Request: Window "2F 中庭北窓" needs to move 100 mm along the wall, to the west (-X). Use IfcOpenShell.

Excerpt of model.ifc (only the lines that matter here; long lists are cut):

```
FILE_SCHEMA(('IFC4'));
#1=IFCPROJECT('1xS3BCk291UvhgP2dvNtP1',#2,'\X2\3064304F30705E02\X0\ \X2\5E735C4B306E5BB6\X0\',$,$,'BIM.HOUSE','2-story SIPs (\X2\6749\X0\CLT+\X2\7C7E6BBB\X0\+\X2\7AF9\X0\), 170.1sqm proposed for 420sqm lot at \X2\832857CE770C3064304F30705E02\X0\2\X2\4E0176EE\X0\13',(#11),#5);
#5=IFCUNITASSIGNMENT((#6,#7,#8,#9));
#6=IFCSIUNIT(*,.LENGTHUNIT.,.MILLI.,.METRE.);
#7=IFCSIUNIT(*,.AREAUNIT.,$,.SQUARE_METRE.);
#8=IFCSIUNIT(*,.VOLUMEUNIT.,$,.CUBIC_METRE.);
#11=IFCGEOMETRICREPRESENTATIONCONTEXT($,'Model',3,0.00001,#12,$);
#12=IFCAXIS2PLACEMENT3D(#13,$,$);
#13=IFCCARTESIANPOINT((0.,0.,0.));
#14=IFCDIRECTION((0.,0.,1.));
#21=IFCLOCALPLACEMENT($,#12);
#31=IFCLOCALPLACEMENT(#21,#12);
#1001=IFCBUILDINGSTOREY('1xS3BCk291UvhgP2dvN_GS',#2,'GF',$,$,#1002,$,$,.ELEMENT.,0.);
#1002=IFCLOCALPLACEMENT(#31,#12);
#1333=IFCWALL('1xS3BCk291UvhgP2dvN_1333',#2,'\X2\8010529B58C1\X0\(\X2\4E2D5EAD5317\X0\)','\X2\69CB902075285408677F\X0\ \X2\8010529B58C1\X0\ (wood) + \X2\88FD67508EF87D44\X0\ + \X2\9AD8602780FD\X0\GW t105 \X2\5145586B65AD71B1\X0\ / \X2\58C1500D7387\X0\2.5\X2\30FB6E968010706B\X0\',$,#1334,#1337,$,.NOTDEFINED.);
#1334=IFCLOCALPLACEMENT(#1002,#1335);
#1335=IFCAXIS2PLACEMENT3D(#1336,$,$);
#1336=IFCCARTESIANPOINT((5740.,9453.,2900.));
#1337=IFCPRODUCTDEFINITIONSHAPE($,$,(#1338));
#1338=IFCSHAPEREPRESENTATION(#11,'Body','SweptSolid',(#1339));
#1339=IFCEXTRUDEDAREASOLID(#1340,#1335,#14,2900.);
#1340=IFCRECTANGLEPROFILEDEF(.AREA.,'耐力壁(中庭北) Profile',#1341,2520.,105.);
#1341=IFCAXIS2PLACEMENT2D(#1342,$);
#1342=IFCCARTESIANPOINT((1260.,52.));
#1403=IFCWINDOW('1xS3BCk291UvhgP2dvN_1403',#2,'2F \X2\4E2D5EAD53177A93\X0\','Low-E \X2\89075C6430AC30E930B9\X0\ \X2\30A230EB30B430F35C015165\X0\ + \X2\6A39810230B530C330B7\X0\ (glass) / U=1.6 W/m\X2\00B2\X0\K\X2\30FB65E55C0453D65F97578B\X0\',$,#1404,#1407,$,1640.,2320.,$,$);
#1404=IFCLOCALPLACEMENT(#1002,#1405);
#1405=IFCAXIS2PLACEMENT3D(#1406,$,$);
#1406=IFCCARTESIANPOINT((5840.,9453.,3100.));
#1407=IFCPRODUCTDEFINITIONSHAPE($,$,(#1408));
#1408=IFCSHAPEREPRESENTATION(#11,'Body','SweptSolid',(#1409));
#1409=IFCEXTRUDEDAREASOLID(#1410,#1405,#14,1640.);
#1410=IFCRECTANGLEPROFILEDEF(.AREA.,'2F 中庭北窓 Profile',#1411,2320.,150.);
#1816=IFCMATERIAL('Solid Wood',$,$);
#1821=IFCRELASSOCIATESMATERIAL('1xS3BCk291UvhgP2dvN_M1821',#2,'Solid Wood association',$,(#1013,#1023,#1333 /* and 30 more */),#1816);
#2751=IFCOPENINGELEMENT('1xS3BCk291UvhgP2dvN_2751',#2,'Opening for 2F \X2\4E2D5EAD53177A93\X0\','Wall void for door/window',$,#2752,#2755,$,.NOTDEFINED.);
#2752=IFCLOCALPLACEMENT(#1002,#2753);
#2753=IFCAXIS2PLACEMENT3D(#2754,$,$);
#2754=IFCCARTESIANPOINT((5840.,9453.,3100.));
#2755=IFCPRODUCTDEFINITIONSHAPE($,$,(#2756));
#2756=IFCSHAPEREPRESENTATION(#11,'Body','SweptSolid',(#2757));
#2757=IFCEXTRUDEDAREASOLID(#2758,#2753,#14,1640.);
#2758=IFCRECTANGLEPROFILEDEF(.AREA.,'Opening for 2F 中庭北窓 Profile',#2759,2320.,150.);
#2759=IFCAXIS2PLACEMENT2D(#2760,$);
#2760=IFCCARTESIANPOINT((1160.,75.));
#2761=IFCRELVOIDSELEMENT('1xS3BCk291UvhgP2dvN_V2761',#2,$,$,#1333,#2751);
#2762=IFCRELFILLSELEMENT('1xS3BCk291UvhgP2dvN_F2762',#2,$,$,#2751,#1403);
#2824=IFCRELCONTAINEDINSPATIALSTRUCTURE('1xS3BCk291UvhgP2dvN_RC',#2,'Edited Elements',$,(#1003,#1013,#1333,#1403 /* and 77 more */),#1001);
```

```python
import ifcopenshell
import ifcopenshell.api.geometry
import ifcopenshell.util.placement
import ifcopenshell.util.unit

model = ifcopenshell.open("model.ifc")
unit_scale = ifcopenshell.util.unit.calculate_unit_scale(model)

window = model.by_guid("1xS3BCk291UvhgP2dvN_1403")
opening = window.FillsVoids[0].RelatingOpeningElement
wall = opening.VoidsElements[0].RelatingBuildingElement

wall_matrix = ifcopenshell.util.placement.get_local_placement(wall.ObjectPlacement)
shift = wall_matrix[:3, 0] * -0.1 / unit_scale
before = ifcopenshell.util.placement.get_local_placement(window.ObjectPlacement)[:3, 3].copy()

# The window is not placed relative to its opening, so move both.
for product in (opening, window):
    matrix = ifcopenshell.util.placement.get_local_placement(product.ObjectPlacement)
    matrix[:3, 3] += shift
    ifcopenshell.api.geometry.edit_object_placement(model, product=product, matrix=matrix, is_si=False)

after = ifcopenshell.util.placement.get_local_placement(window.ObjectPlacement)[:3, 3]
print("window moved by", (after - before).round(3) + 0.0)

model.write("model_rev.ifc")
```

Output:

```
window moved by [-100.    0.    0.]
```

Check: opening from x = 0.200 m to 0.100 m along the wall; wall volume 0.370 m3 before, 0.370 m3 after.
